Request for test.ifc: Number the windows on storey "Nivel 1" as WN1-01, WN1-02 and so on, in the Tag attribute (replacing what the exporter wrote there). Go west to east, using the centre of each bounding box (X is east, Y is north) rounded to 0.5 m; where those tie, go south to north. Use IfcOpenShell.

First a look at what the model holds.

```python
import ifcopenshell
import ifcopenshell.util.element
import ifcopenshell.util.placement

model = ifcopenshell.open("test.ifc")
print(model.schema)
storey = next(s for s in model.by_type("IfcBuildingStorey") if s.Name == "Nivel 1")
windows = [e for e in ifcopenshell.util.element.get_decomposition(storey) if e.is_a("IfcWindow")]
for e in sorted(windows, key=lambda e: e.id()):
    origin = ifcopenshell.util.placement.get_local_placement(e.ObjectPlacement)[:3, 3]
    print(e.id(), e.Tag, e.Name, origin.round(2) + 0.0, sep=" | ")
```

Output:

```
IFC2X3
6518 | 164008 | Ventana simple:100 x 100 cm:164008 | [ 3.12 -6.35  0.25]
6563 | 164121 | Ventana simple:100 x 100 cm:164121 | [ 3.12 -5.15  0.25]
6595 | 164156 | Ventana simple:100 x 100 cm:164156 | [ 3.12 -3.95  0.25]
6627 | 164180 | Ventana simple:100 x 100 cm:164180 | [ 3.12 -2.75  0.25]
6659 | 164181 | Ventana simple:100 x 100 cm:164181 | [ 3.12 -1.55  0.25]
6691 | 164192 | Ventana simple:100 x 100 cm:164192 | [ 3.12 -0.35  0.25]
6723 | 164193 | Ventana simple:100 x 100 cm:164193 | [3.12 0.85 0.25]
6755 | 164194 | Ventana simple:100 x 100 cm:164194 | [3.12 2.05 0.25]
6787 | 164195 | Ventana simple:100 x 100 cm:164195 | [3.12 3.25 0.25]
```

```python
import ifcopenshell
import ifcopenshell.geom
import ifcopenshell.util.element
import ifcopenshell.util.shape

model = ifcopenshell.open("test.ifc")
settings = ifcopenshell.geom.settings()
settings.set("use-world-coords", True)


def centre(element):
    shape = ifcopenshell.geom.create_shape(settings, element)
    return ifcopenshell.util.shape.get_bbox_centroid(shape.geometry)


storey = next(s for s in model.by_type("IfcBuildingStorey") if s.Name == "Nivel 1")
windows = [e for e in ifcopenshell.util.element.get_decomposition(storey) if e.is_a("IfcWindow")]

# Insertion points can sit at a corner or the storey origin, so sort by the geometry (in metres).
centres = {e: centre(e) for e in windows}
windows.sort(key=lambda e: (round(centres[e][0] / 0.5), centres[e][1]))

for i, e in enumerate(windows, start=1):
    number = f"WN1-{i:02d}"
    e.Tag = number
    print(e.id(), number)

model.write("test_rev.ifc")
```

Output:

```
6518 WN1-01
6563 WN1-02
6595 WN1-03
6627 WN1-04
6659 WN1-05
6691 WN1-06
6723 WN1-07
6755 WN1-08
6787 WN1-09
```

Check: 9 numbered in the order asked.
